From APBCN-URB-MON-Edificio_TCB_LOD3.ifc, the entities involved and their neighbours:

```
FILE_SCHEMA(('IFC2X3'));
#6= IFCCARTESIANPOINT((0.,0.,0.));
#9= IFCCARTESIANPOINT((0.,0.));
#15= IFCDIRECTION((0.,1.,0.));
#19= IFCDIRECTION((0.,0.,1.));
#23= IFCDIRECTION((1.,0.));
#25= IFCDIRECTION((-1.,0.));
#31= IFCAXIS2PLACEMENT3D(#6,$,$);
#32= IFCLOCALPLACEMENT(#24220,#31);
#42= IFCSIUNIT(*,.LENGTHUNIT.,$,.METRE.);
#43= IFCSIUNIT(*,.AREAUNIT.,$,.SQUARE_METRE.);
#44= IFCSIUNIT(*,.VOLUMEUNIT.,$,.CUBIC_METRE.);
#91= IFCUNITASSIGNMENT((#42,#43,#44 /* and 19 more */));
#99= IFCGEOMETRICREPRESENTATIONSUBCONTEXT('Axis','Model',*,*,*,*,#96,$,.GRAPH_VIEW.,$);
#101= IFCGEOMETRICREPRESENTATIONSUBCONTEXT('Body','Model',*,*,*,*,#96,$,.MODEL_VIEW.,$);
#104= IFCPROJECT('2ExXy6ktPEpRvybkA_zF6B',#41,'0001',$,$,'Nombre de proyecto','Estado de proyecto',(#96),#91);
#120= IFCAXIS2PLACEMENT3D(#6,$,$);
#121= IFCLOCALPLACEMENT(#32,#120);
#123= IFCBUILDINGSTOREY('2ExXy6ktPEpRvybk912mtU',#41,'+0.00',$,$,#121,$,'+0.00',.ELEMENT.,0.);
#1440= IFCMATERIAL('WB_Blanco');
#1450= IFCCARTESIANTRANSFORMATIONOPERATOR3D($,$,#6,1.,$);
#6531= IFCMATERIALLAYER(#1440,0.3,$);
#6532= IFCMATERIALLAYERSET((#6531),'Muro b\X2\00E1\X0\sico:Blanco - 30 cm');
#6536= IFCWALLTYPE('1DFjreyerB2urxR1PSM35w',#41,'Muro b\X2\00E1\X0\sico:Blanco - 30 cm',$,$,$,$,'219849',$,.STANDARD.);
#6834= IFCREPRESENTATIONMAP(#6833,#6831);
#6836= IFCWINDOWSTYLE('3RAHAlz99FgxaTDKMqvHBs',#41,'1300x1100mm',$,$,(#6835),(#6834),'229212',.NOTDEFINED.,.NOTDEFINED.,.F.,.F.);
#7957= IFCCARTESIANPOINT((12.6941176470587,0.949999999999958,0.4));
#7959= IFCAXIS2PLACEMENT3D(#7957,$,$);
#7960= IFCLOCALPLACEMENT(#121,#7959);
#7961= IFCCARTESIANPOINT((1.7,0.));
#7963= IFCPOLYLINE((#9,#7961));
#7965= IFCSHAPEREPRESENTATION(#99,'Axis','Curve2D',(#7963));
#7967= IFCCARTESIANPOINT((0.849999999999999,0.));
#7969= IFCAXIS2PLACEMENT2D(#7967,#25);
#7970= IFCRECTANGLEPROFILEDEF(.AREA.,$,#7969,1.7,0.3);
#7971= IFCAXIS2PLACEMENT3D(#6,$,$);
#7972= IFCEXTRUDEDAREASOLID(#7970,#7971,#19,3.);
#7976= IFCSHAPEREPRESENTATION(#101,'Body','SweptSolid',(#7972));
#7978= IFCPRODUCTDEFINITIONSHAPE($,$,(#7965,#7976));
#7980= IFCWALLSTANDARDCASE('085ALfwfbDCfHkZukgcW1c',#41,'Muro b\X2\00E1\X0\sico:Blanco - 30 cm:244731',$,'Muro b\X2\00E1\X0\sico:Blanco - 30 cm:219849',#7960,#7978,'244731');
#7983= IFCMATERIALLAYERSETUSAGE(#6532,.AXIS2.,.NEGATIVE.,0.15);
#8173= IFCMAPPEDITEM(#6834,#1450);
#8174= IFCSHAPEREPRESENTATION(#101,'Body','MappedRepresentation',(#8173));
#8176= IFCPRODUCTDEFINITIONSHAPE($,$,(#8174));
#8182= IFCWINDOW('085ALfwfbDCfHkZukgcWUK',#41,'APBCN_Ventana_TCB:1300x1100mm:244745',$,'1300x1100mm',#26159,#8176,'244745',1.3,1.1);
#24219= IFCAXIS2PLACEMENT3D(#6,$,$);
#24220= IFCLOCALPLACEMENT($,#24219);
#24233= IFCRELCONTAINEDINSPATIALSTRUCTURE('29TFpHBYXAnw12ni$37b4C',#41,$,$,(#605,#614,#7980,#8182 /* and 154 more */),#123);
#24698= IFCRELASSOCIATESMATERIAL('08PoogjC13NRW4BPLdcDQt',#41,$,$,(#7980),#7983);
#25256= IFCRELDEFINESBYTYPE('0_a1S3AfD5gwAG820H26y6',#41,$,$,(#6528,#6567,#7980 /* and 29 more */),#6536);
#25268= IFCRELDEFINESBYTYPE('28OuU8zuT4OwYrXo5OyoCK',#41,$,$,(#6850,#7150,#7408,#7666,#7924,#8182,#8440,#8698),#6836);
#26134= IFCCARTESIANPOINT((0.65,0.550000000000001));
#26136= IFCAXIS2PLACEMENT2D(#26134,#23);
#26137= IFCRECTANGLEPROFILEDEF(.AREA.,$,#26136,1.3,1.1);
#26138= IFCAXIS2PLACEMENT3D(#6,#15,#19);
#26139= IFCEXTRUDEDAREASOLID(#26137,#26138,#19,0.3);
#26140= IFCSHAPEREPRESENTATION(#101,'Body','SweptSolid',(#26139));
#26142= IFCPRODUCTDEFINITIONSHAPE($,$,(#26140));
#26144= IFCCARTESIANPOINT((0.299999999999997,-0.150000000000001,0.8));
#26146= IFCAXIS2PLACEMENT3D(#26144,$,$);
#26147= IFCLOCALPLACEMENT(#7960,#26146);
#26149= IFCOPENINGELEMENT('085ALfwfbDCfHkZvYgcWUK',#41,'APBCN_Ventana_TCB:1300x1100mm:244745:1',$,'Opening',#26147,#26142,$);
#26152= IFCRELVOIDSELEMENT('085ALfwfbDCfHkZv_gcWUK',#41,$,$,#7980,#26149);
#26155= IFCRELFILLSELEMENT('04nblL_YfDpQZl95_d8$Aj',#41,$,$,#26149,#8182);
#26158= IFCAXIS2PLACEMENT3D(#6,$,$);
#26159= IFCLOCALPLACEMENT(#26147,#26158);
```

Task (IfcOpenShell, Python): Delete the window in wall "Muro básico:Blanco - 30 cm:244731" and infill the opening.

```python
import ifcopenshell
import ifcopenshell.api.feature
import ifcopenshell.api.root
import ifcopenshell.geom
import ifcopenshell.util.shape

model = ifcopenshell.open("APBCN-URB-MON-Edificio_TCB_LOD3.ifc")
settings = ifcopenshell.geom.settings()


def volume(element):
    """Net volume in cubic metres, openings subtracted."""
    shape = ifcopenshell.geom.create_shape(settings, element)
    return ifcopenshell.util.shape.get_volume(shape.geometry)


window = model.by_guid("085ALfwfbDCfHkZukgcWUK")
opening = window.FillsVoids[0].RelatingOpeningElement
wall = opening.VoidsElements[0].RelatingBuildingElement
before = volume(wall)

ifcopenshell.api.root.remove_product(model, product=window)
ifcopenshell.api.feature.remove_feature(model, feature=opening)

after = volume(wall)

print(f"wall volume {before:.3f} -> {after:.3f} m3")

model.write("APBCN-URB-MON-Edificio_TCB_LOD3_v2.ifc")
```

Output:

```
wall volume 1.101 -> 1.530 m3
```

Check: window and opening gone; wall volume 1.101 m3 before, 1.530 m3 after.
